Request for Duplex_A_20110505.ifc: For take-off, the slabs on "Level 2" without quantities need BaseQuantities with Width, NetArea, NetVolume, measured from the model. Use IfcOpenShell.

First a look at what the model holds.

```python
import ifcopenshell
import ifcopenshell.util.element
import ifcopenshell.util.unit

model = ifcopenshell.open("Duplex_A_20110505.ifc")
print(model.schema)
for unit_type in ("LENGTHUNIT", "AREAUNIT", "VOLUMEUNIT"):
    print(unit_type, ifcopenshell.util.unit.calculate_unit_scale(model, unit_type))
storey = next(s for s in model.by_type("IfcBuildingStorey") if s.Name == "Level 2")
slabs = [e for e in ifcopenshell.util.element.get_decomposition(storey) if e.is_a("IfcSlab")]
for e in sorted(slabs, key=lambda e: e.id()):
    print(e.id(), e.is_a(), e.Name, list(ifcopenshell.util.element.get_psets(e, qtos_only=True)), sep=" | ")
```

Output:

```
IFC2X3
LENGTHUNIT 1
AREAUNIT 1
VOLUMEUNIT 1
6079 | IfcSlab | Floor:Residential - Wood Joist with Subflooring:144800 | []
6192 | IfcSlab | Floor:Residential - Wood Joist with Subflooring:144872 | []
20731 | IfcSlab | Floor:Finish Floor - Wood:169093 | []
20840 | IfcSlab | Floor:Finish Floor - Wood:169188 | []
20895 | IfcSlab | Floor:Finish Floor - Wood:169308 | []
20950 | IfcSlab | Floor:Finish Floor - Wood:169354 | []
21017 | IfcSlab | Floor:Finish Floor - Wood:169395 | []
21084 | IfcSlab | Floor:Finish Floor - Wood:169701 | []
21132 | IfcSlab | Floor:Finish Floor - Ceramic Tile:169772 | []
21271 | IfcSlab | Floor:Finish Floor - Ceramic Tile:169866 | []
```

```python
import ifcopenshell
import ifcopenshell.api.pset
import ifcopenshell.geom
import ifcopenshell.util.element
import ifcopenshell.util.shape
import ifcopenshell.util.unit

model = ifcopenshell.open("Duplex_A_20110505.ifc")
unit_scale = ifcopenshell.util.unit.calculate_unit_scale(model)
area_scale = ifcopenshell.util.unit.calculate_unit_scale(model, "AREAUNIT")
volume_scale = ifcopenshell.util.unit.calculate_unit_scale(model, "VOLUMEUNIT")
settings = ifcopenshell.geom.settings()

storey = next(s for s in model.by_type("IfcBuildingStorey") if s.Name == "Level 2")
slabs = [e for e in ifcopenshell.util.element.get_decomposition(storey) if e.is_a("IfcSlab")]

for e in sorted(slabs, key=lambda e: e.id()):
    if ifcopenshell.util.element.get_psets(e, qtos_only=True, should_inherit=False):
        continue
    # Geometry comes back in metres, in the element's own axes.
    shape = ifcopenshell.geom.create_shape(settings, e)
    values = {
        "Width": ifcopenshell.util.shape.get_z(shape.geometry) / unit_scale,
        "NetArea": ifcopenshell.util.shape.get_footprint_area(shape.geometry) / area_scale,
        "NetVolume": ifcopenshell.util.shape.get_volume(shape.geometry) / volume_scale,
    }
    qto = ifcopenshell.api.pset.add_qto(model, product=e, name="BaseQuantities")
    ifcopenshell.api.pset.edit_qto(model, qto=qto, properties=values)
    print(e.id(), {k: round(v, 3) for k, v in values.items()})

model.write("Duplex_A_20110505_v2.ifc")
```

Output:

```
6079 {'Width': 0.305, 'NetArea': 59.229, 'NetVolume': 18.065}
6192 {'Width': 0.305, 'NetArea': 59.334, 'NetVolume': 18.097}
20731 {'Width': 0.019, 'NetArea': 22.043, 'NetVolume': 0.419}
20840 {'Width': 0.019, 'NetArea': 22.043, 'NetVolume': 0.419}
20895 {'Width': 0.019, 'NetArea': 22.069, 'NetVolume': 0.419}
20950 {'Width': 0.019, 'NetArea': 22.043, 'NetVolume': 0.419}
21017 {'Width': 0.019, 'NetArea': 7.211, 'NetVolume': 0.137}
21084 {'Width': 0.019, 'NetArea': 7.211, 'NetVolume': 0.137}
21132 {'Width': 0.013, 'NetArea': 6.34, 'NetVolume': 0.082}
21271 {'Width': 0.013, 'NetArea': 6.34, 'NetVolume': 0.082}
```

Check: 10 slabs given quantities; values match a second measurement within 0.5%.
